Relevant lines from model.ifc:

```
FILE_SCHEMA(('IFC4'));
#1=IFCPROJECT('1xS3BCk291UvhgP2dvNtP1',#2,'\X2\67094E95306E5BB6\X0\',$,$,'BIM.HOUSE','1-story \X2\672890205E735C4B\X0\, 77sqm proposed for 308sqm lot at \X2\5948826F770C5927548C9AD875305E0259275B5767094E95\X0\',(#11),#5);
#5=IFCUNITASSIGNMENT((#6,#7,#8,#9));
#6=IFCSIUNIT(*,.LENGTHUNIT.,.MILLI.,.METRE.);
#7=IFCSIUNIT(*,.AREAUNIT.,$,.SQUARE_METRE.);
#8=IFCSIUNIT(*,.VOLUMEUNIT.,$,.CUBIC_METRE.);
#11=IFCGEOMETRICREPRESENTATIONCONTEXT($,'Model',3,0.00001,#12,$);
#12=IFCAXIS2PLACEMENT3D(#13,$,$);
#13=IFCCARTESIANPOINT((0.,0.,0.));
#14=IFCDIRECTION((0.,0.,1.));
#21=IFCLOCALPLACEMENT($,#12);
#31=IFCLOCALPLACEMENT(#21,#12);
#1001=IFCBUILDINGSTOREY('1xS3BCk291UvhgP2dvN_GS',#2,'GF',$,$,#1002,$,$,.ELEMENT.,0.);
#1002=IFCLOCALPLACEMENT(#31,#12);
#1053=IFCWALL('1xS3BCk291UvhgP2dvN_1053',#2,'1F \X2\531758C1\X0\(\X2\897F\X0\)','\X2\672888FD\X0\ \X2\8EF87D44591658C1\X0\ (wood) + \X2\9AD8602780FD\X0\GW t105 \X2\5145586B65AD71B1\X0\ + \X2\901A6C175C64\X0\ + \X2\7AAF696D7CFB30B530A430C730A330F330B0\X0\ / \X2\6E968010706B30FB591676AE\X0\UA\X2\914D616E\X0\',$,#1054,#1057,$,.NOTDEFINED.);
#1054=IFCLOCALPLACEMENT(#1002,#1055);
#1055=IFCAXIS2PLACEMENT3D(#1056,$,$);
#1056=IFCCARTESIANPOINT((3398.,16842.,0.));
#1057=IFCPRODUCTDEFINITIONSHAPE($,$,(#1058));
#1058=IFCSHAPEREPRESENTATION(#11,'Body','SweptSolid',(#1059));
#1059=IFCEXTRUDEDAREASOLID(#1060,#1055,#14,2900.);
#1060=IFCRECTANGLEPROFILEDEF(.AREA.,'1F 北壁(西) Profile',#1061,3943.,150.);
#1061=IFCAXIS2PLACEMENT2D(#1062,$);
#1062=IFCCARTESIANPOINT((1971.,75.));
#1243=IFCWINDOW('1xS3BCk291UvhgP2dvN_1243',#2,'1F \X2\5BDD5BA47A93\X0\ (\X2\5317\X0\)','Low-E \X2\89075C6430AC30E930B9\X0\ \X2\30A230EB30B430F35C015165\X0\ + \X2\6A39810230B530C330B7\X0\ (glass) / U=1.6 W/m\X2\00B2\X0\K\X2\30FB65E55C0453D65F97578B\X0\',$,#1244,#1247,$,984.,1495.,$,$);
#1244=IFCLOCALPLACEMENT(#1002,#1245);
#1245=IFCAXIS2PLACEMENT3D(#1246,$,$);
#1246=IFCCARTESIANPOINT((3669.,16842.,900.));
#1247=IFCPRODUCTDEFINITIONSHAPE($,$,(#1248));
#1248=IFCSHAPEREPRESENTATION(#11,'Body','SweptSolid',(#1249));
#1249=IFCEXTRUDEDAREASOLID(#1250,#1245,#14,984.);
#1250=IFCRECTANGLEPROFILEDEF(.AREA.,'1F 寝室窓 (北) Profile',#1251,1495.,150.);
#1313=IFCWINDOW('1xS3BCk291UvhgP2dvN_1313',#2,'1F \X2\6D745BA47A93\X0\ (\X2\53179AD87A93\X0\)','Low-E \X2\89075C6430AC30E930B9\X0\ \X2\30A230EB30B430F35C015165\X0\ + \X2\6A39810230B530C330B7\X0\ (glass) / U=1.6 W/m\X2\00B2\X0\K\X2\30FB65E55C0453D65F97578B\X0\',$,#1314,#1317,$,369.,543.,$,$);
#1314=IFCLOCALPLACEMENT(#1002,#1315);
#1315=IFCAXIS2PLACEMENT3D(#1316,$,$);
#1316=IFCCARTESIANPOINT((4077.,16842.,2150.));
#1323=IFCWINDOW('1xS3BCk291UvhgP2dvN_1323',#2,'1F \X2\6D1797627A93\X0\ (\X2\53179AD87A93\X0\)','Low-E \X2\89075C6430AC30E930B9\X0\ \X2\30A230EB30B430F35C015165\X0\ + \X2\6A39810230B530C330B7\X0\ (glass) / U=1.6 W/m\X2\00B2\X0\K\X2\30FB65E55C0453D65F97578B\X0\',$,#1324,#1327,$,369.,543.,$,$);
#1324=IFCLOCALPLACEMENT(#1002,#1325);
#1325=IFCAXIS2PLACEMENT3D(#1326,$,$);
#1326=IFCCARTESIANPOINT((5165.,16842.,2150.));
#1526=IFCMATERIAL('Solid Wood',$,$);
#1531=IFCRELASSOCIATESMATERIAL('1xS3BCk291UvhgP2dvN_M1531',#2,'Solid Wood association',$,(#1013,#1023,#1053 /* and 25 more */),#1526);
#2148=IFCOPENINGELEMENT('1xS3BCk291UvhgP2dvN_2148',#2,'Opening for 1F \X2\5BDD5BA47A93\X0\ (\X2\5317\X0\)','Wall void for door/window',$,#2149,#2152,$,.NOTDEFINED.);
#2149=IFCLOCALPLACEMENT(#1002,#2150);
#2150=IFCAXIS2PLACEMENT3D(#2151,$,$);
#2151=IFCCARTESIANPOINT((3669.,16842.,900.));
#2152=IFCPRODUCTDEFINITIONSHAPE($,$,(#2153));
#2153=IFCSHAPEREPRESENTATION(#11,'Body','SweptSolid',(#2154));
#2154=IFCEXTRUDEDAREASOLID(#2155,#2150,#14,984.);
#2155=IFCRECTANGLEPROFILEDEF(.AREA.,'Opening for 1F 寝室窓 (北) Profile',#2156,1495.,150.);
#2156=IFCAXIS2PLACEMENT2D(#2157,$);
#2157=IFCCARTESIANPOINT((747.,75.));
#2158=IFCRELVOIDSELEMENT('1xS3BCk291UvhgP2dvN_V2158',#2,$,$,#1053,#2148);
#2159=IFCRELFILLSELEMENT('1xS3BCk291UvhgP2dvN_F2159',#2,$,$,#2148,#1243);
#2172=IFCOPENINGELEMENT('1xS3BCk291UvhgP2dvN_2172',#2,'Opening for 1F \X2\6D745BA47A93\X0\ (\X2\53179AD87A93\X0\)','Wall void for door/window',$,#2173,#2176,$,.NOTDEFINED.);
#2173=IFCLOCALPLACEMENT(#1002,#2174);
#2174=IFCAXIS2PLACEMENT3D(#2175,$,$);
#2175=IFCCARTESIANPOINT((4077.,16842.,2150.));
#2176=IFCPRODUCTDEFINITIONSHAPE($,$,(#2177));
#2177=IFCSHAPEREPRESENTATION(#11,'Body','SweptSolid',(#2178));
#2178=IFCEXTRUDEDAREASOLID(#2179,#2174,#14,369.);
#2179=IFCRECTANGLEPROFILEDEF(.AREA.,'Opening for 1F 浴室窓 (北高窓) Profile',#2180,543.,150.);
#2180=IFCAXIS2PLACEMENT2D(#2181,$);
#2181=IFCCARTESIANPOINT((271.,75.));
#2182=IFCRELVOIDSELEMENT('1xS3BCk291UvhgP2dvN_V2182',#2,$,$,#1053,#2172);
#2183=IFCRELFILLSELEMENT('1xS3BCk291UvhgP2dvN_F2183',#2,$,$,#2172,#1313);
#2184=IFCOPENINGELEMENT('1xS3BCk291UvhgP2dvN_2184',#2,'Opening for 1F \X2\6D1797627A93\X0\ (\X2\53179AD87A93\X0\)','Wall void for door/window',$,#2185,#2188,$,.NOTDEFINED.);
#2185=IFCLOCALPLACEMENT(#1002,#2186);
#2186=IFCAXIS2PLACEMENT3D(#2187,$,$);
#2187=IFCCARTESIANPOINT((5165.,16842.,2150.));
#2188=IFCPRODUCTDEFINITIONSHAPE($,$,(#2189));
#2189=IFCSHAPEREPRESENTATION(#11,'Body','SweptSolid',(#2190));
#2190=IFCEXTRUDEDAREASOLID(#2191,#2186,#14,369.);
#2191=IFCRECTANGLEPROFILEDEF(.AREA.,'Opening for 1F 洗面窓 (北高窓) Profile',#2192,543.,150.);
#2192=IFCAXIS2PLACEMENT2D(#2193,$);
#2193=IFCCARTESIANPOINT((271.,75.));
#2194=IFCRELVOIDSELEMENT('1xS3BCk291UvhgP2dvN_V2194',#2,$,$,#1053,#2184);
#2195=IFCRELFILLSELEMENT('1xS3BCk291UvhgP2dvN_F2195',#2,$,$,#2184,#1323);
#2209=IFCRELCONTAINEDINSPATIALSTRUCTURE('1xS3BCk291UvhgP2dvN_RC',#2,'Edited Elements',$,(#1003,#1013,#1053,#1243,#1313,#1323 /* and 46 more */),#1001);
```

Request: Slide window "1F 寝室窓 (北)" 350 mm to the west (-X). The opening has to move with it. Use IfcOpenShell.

```python
import ifcopenshell
import ifcopenshell.api.geometry
import ifcopenshell.util.placement

model = ifcopenshell.open("model.ifc")

window = model.by_guid("1xS3BCk291UvhgP2dvN_1243")
opening = window.FillsVoids[0].RelatingOpeningElement
wall = opening.VoidsElements[0].RelatingBuildingElement

wall_matrix = ifcopenshell.util.placement.get_local_placement(wall.ObjectPlacement)
shift = wall_matrix[:3, 0] * -350.0
before = ifcopenshell.util.placement.get_local_placement(window.ObjectPlacement)[:3, 3].copy()

# The window is not placed relative to its opening, so move both.
for product in (opening, window):
    matrix = ifcopenshell.util.placement.get_local_placement(product.ObjectPlacement)
    matrix[:3, 3] += shift
    ifcopenshell.api.geometry.edit_object_placement(model, product=product, matrix=matrix, is_si=False)

after = ifcopenshell.util.placement.get_local_placement(window.ObjectPlacement)[:3, 3]
print("window moved by", (after - before).round(3) + 0.0)

model.write("model_v2.ifc")
```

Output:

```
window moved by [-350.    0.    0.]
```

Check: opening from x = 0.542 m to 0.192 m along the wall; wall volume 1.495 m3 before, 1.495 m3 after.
